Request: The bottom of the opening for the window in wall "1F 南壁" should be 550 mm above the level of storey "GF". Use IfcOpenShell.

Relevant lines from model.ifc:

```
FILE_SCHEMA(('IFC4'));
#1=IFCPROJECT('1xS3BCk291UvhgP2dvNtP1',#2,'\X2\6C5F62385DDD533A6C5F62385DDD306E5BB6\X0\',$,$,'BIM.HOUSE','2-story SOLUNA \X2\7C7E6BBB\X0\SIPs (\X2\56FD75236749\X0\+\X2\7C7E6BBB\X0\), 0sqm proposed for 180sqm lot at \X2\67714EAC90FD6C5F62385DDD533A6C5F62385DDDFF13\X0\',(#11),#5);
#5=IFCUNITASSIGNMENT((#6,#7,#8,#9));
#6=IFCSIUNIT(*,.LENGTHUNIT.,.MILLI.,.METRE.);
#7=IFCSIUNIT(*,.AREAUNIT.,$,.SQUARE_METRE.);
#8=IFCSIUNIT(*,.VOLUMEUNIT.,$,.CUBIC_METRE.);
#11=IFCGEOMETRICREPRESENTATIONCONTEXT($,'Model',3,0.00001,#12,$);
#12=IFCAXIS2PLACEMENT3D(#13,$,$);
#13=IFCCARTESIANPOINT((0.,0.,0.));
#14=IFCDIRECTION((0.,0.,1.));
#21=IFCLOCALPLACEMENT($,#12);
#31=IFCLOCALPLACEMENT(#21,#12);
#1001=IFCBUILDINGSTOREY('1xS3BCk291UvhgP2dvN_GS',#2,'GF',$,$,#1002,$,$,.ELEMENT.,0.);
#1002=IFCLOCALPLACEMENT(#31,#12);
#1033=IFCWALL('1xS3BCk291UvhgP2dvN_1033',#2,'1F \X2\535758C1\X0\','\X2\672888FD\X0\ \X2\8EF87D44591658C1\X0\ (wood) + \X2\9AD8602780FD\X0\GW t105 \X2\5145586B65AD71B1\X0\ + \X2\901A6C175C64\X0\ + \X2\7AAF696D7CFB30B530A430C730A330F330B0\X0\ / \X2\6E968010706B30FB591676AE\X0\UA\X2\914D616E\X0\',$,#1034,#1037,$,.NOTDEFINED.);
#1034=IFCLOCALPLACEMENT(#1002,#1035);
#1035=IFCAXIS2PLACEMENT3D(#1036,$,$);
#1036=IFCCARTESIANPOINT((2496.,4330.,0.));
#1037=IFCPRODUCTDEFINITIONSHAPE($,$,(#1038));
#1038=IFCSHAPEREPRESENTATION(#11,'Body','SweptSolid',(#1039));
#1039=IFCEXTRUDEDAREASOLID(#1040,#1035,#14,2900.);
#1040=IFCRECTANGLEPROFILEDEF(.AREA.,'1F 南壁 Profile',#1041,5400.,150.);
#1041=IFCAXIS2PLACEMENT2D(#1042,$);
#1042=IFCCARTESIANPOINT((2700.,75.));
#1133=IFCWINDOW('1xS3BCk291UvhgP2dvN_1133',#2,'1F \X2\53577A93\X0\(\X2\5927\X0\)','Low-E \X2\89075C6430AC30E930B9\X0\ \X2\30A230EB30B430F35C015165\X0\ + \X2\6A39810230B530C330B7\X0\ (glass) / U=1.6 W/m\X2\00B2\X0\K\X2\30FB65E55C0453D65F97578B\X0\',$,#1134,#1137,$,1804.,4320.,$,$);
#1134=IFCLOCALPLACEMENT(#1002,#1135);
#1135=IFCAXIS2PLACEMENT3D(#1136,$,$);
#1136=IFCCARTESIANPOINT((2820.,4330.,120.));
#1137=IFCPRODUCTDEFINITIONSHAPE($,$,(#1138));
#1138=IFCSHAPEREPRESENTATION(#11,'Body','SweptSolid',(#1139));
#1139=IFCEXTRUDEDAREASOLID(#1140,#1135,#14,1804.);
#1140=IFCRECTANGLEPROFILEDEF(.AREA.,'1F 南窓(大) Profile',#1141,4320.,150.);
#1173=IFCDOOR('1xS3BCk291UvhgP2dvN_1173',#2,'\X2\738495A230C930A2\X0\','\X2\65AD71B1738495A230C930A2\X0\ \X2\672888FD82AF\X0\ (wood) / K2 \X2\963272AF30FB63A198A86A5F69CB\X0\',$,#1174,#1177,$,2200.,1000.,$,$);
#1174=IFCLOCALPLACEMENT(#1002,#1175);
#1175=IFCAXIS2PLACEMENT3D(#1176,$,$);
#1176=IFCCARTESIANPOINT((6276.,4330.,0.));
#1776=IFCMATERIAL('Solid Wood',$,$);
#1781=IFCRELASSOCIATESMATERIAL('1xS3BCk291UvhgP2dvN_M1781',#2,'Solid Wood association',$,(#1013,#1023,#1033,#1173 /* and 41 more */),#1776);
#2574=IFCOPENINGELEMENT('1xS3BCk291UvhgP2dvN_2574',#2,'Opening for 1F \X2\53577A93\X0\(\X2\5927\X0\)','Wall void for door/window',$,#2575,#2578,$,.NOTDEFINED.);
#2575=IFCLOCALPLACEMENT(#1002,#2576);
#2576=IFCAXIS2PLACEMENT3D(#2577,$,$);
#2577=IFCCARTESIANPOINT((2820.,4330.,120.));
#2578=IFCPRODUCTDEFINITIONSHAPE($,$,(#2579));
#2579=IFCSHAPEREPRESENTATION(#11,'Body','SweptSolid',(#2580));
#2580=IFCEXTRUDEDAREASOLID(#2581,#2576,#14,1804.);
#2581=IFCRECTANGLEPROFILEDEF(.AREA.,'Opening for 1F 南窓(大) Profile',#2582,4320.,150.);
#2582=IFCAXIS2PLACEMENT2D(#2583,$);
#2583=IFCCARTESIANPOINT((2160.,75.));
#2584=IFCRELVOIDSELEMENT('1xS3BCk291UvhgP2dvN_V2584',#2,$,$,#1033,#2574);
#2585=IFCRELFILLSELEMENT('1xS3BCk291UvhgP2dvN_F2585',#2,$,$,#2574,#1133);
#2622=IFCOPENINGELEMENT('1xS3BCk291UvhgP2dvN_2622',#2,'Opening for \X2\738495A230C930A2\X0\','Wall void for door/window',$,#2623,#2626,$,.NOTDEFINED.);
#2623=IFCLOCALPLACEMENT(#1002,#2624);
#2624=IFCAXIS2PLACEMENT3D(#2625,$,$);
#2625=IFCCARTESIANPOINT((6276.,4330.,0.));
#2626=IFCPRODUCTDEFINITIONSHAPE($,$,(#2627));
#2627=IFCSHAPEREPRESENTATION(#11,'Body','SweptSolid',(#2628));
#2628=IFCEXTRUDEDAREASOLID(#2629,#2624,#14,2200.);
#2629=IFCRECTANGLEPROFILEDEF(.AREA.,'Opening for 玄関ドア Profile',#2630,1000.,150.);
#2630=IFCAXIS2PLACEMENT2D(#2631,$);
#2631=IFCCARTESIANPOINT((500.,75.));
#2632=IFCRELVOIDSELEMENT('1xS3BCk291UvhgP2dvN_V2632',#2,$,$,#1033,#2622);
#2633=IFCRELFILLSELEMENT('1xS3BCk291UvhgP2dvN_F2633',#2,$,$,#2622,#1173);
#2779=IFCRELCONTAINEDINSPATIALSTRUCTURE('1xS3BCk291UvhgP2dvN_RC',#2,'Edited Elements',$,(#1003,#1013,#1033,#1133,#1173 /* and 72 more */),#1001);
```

```python
import numpy as np
import ifcopenshell
import ifcopenshell.api.geometry
import ifcopenshell.geom
import ifcopenshell.util.element
import ifcopenshell.util.placement
import ifcopenshell.util.shape
import ifcopenshell.util.unit

model = ifcopenshell.open("model.ifc")
unit_scale = ifcopenshell.util.unit.calculate_unit_scale(model)

window = model.by_guid("1xS3BCk291UvhgP2dvN_1133")
opening = window.FillsVoids[0].RelatingOpeningElement
storey = ifcopenshell.util.element.get_container(window, ifc_class="IfcBuildingStorey")
level = ifcopenshell.util.placement.get_local_placement(storey.ObjectPlacement)[2, 3]

# The opening's origin need not be at the sill, so measure its lowest point.
shape = ifcopenshell.geom.create_shape(ifcopenshell.geom.settings(), opening)
bottom = ifcopenshell.util.shape.get_shape_bottom_elevation(shape, shape.geometry) / unit_scale
dz = level + 550.0 - bottom

shift = np.array([0.0, 0.0, dz])
# The window is not placed relative to its opening, so move both.
for product in (opening, window):
    matrix = ifcopenshell.util.placement.get_local_placement(product.ObjectPlacement)
    matrix[:3, 3] += shift
    ifcopenshell.api.geometry.edit_object_placement(model, product=product, matrix=matrix, is_si=False)

print(f"moved by {dz * unit_scale:+.3f} m")

model.write("model_rev.ifc")
```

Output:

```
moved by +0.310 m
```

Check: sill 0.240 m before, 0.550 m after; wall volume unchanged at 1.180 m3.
